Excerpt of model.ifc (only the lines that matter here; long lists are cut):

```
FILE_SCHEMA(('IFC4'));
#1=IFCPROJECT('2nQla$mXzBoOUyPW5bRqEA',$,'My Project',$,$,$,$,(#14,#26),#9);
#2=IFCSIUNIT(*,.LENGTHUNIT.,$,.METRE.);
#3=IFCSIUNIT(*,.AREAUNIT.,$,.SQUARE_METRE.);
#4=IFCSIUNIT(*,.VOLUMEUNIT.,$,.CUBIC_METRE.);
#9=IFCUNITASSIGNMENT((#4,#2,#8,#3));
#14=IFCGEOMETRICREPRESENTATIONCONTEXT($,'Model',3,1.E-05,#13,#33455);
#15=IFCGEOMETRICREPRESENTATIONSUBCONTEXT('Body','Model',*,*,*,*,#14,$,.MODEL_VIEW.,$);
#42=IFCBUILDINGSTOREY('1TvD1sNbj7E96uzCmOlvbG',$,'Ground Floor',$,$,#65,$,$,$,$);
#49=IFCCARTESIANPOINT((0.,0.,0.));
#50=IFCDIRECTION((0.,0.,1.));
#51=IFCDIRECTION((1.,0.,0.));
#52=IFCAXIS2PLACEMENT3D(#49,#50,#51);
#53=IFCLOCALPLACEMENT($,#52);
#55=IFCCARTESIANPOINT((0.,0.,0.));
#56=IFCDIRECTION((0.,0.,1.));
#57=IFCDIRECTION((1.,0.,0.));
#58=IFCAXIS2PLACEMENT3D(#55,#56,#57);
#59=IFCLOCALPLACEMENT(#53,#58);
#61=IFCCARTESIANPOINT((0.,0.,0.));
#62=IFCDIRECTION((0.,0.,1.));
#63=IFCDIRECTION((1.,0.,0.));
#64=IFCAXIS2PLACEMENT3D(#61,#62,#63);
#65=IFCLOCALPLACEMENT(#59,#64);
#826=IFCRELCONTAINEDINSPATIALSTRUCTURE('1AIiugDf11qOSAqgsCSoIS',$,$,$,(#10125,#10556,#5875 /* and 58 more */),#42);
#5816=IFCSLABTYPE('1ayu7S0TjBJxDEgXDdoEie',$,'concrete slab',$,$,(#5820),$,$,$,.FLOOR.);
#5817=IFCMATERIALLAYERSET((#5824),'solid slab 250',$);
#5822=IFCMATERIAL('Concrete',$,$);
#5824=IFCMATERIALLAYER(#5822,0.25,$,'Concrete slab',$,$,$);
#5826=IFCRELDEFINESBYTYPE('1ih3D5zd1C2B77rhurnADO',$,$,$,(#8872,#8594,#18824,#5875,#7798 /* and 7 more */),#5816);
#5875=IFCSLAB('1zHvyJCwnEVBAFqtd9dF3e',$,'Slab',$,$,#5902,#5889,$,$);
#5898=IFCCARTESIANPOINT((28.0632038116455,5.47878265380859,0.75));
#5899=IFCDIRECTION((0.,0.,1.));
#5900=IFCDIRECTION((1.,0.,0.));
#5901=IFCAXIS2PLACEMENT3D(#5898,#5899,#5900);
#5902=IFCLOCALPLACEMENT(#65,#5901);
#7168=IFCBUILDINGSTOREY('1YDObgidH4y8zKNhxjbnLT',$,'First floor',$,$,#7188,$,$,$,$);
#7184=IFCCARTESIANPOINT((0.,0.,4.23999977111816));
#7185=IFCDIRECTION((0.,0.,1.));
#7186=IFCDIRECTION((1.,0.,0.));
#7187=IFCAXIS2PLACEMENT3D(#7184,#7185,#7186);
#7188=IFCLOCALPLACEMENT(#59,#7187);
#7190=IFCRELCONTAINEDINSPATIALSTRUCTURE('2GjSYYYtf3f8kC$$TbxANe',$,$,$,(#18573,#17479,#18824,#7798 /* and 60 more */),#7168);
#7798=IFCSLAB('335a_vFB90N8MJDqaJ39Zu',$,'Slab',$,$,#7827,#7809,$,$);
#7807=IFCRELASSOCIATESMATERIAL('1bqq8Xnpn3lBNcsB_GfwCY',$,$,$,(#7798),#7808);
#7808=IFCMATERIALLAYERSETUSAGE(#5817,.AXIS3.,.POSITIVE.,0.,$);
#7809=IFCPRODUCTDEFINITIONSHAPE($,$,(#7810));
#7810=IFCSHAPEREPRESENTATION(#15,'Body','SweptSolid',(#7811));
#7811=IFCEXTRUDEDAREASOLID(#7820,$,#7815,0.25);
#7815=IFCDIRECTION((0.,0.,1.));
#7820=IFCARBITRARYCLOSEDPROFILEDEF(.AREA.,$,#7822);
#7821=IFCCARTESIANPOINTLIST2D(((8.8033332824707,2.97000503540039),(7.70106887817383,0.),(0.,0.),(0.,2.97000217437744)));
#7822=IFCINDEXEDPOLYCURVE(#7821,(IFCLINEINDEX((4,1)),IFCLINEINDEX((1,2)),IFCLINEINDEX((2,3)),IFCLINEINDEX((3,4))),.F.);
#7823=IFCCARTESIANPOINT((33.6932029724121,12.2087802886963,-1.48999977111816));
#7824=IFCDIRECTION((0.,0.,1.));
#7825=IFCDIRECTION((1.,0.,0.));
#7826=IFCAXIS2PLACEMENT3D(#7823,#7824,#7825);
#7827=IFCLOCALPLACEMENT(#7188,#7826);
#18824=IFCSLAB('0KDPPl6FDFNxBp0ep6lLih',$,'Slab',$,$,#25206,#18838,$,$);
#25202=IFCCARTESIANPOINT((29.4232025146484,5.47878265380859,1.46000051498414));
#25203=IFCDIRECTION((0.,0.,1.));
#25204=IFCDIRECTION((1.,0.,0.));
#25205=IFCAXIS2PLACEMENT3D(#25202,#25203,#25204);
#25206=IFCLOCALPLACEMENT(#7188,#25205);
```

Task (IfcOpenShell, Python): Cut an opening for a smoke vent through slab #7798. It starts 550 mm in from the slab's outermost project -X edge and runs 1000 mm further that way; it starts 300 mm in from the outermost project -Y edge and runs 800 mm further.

```python
import numpy as np
import ifcopenshell
import ifcopenshell.api.feature
import ifcopenshell.api.geometry
import ifcopenshell.api.root
import ifcopenshell.geom
import ifcopenshell.util.placement
import ifcopenshell.util.representation
import ifcopenshell.util.shape
import ifcopenshell.util.unit

model = ifcopenshell.open("model.ifc")
unit_scale = ifcopenshell.util.unit.calculate_unit_scale(model)
settings = ifcopenshell.geom.settings()


def volume(element):
    """Net volume in cubic metres, openings subtracted."""
    shape = ifcopenshell.geom.create_shape(settings, element)
    return ifcopenshell.util.shape.get_volume(shape.geometry)


slab = model.by_guid("335a_vFB90N8MJDqaJ39Zu")
before = volume(slab)

# Extent in the slab's own axes, in metres. The edges named are its -X and -Y sides.
slab_shape = ifcopenshell.geom.create_shape(settings, slab)
vertices = ifcopenshell.util.shape.get_vertices(slab_shape.geometry)
x_min, y_min, bottom = vertices.min(axis=0)
top = vertices[:, 2].max()

opening = ifcopenshell.api.root.create_entity(model, ifc_class="IfcOpeningElement", name="Smoke vent opening", predefined_type="OPENING")
context = ifcopenshell.util.representation.get_context(model, "Model", "Body", "MODEL_VIEW")
width, depth = 1, 0.8
outline = [(0.0, 0.0), (width, 0.0), (width, depth), (0.0, depth), (0.0, 0.0)]
# Overshoot both faces by 50 mm so the cut is clean.
shape = ifcopenshell.api.geometry.add_slab_representation(
    model, context=context, depth=top - bottom + 0.1, polyline=outline
)
ifcopenshell.api.geometry.assign_representation(model, product=opening, representation=shape)

matrix = ifcopenshell.util.placement.get_local_placement(slab.ObjectPlacement)
matrix[:, 3] = matrix @ np.append(np.array([x_min + 0.55, y_min + 0.3, bottom - 0.05]) / unit_scale, 1.0)
ifcopenshell.api.geometry.edit_object_placement(model, product=opening, matrix=matrix, is_si=False)
ifcopenshell.api.feature.add_feature(model, feature=opening, element=slab)

after = volume(slab)

print(f"slab volume {before:.3f} -> {after:.3f} m3")

model.write("model_rev.ifc")
```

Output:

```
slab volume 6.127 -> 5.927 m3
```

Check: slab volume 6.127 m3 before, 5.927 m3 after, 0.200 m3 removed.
